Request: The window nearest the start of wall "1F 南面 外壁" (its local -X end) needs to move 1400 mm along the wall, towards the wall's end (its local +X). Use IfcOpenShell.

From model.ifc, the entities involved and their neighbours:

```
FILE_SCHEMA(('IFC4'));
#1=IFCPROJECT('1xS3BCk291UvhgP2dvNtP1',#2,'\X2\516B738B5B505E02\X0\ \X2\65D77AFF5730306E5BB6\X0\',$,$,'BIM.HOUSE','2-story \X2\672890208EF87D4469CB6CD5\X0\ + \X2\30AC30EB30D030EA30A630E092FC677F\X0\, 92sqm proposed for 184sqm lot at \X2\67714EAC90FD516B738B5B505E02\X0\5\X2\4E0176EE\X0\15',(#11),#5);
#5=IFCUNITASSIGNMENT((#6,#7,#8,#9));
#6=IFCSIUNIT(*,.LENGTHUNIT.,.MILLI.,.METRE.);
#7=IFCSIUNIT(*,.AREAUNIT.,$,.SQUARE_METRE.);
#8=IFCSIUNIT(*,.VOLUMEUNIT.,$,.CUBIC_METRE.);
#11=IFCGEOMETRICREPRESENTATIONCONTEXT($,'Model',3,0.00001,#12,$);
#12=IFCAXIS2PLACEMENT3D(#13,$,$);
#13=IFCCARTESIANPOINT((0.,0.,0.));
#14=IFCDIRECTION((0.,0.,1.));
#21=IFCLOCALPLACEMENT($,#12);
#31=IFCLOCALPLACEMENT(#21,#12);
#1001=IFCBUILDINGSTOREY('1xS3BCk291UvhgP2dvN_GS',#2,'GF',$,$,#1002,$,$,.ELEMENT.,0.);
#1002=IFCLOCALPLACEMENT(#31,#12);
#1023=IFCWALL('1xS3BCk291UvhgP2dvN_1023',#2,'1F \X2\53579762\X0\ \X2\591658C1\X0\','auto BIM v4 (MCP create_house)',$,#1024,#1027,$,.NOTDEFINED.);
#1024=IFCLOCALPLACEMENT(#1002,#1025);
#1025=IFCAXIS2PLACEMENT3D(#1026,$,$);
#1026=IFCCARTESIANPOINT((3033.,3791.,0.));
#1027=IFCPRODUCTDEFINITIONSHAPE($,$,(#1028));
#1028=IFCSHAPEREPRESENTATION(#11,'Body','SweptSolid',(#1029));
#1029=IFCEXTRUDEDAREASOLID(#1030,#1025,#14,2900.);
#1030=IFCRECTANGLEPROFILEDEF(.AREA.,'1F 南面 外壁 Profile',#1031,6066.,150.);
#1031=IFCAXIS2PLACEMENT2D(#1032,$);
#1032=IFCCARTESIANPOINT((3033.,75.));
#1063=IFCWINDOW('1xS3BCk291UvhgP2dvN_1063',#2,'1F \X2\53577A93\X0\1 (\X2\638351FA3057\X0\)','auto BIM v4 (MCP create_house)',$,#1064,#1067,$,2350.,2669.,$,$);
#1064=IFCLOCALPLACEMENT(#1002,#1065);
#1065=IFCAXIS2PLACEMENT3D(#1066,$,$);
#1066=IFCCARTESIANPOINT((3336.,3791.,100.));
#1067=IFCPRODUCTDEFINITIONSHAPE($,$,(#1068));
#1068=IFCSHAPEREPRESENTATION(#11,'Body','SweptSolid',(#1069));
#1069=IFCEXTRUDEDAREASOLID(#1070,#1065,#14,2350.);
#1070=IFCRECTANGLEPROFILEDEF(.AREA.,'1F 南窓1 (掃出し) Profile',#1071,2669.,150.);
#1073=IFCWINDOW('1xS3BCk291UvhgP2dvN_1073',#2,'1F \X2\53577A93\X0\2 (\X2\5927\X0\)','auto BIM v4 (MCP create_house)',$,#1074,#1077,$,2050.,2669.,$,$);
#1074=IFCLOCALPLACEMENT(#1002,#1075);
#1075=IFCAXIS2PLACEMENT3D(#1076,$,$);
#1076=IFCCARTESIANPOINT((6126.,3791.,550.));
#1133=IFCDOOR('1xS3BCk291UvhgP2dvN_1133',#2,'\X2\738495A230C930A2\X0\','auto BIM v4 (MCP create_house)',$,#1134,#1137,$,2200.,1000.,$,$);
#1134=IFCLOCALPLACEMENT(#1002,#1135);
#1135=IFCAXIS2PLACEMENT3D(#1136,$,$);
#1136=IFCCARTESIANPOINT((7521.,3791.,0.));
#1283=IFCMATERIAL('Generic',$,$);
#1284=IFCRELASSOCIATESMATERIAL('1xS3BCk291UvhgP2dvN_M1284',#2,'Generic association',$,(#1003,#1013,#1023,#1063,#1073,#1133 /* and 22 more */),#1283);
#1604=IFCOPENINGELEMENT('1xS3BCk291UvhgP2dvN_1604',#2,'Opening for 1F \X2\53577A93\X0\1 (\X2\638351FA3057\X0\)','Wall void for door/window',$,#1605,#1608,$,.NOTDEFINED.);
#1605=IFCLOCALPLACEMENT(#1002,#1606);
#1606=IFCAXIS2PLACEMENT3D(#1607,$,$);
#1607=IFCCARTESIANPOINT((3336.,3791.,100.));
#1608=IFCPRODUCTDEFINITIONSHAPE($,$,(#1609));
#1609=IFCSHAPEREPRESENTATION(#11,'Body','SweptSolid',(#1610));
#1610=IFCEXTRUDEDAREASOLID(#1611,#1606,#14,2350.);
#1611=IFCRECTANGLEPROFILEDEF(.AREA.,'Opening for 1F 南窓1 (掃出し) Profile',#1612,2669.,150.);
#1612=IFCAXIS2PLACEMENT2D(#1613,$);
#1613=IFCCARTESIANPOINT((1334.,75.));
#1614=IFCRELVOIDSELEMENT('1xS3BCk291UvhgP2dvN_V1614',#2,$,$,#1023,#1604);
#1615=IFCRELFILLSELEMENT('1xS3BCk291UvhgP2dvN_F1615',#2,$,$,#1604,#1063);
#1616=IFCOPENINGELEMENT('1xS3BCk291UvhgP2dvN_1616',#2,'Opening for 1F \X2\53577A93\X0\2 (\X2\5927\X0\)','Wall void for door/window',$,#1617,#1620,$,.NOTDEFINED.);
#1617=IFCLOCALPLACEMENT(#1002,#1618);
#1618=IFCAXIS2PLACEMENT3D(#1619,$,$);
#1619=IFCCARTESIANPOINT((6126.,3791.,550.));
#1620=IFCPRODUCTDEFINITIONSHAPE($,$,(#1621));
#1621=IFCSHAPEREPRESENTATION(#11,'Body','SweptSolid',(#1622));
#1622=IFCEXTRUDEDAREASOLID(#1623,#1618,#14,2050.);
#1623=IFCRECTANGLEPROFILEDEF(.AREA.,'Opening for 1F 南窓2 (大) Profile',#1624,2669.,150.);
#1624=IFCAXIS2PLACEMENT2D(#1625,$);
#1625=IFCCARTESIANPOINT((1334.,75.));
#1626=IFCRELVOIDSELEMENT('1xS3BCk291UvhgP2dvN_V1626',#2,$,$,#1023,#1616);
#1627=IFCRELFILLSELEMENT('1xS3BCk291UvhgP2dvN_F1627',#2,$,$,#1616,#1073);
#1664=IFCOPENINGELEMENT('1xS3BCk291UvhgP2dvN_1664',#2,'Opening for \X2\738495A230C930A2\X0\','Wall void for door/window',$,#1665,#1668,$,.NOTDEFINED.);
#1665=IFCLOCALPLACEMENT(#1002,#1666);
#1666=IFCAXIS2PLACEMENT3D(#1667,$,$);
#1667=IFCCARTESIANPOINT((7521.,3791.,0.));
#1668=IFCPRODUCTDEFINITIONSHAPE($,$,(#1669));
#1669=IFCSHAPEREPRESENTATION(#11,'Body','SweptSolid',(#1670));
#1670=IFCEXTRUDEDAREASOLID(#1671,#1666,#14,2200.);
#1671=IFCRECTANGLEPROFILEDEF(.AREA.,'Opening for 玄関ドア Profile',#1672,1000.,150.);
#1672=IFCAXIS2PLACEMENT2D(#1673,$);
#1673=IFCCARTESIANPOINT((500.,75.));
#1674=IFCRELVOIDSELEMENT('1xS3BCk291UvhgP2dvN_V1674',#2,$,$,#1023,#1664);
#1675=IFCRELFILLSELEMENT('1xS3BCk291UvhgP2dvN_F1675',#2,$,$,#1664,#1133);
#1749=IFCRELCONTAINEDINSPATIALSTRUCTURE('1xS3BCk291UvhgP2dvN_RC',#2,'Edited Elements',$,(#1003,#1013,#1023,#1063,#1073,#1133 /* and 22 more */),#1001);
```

```python
import ifcopenshell
import ifcopenshell.api.geometry
import ifcopenshell.util.placement
import ifcopenshell.util.unit

model = ifcopenshell.open("model.ifc")
unit_scale = ifcopenshell.util.unit.calculate_unit_scale(model)

window = model.by_id(1063)
opening = window.FillsVoids[0].RelatingOpeningElement
wall = opening.VoidsElements[0].RelatingBuildingElement

wall_matrix = ifcopenshell.util.placement.get_local_placement(wall.ObjectPlacement)
shift = wall_matrix[:3, 0] * 1.4 / unit_scale
before = ifcopenshell.util.placement.get_local_placement(window.ObjectPlacement)[:3, 3].copy()

# The window is not placed relative to its opening, so move both.
for product in (opening, window):
    matrix = ifcopenshell.util.placement.get_local_placement(product.ObjectPlacement)
    matrix[:3, 3] += shift
    ifcopenshell.api.geometry.edit_object_placement(model, product=product, matrix=matrix, is_si=False)

after = ifcopenshell.util.placement.get_local_placement(window.ObjectPlacement)[:3, 3]
print("window moved by", (after - before).round(3) + 0.0)

model.write("model_edited.ifc")
```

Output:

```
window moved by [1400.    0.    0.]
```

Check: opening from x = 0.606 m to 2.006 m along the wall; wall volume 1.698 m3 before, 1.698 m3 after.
